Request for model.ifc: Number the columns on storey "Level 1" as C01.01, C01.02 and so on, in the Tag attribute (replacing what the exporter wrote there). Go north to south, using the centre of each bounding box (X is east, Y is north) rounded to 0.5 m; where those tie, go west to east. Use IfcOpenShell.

First a look at what the model holds.

```python
import ifcopenshell
import ifcopenshell.util.element
import ifcopenshell.util.placement

model = ifcopenshell.open("model.ifc")
print(model.schema)
storey = next(s for s in model.by_type("IfcBuildingStorey") if s.Name == "Level 1")
columns = [e for e in ifcopenshell.util.element.get_decomposition(storey) if e.is_a("IfcColumn")]
for e in sorted(columns, key=lambda e: e.id()):
    origin = ifcopenshell.util.placement.get_local_placement(e.ObjectPlacement)[:3, 3]
    print(e.id(), e.Tag, e.Name, origin.round(2) + 0.0, sep=" | ")
```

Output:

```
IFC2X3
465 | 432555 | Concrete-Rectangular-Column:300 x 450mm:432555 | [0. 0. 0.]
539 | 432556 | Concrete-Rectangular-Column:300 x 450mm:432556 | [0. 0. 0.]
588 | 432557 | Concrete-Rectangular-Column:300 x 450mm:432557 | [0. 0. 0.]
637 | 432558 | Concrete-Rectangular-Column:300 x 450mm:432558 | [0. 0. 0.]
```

```python
import ifcopenshell
import ifcopenshell.geom
import ifcopenshell.util.element
import ifcopenshell.util.shape

model = ifcopenshell.open("model.ifc")
settings = ifcopenshell.geom.settings()
settings.set("use-world-coords", True)


def centre(element):
    shape = ifcopenshell.geom.create_shape(settings, element)
    return ifcopenshell.util.shape.get_bbox_centroid(shape.geometry)


storey = next(s for s in model.by_type("IfcBuildingStorey") if s.Name == "Level 1")
columns = [e for e in ifcopenshell.util.element.get_decomposition(storey) if e.is_a("IfcColumn")]

# Insertion points can sit at a corner or the storey origin, so sort by the geometry (in metres).
centres = {e: centre(e) for e in columns}
columns.sort(key=lambda e: (-round(centres[e][1] / 0.5), centres[e][0]))

for i, e in enumerate(columns, start=1):
    number = f"C01.{i:02d}"
    e.Tag = number
    print(e.id(), number)

model.write("model_edited.ifc")
```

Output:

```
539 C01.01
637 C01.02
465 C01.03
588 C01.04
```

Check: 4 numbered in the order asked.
